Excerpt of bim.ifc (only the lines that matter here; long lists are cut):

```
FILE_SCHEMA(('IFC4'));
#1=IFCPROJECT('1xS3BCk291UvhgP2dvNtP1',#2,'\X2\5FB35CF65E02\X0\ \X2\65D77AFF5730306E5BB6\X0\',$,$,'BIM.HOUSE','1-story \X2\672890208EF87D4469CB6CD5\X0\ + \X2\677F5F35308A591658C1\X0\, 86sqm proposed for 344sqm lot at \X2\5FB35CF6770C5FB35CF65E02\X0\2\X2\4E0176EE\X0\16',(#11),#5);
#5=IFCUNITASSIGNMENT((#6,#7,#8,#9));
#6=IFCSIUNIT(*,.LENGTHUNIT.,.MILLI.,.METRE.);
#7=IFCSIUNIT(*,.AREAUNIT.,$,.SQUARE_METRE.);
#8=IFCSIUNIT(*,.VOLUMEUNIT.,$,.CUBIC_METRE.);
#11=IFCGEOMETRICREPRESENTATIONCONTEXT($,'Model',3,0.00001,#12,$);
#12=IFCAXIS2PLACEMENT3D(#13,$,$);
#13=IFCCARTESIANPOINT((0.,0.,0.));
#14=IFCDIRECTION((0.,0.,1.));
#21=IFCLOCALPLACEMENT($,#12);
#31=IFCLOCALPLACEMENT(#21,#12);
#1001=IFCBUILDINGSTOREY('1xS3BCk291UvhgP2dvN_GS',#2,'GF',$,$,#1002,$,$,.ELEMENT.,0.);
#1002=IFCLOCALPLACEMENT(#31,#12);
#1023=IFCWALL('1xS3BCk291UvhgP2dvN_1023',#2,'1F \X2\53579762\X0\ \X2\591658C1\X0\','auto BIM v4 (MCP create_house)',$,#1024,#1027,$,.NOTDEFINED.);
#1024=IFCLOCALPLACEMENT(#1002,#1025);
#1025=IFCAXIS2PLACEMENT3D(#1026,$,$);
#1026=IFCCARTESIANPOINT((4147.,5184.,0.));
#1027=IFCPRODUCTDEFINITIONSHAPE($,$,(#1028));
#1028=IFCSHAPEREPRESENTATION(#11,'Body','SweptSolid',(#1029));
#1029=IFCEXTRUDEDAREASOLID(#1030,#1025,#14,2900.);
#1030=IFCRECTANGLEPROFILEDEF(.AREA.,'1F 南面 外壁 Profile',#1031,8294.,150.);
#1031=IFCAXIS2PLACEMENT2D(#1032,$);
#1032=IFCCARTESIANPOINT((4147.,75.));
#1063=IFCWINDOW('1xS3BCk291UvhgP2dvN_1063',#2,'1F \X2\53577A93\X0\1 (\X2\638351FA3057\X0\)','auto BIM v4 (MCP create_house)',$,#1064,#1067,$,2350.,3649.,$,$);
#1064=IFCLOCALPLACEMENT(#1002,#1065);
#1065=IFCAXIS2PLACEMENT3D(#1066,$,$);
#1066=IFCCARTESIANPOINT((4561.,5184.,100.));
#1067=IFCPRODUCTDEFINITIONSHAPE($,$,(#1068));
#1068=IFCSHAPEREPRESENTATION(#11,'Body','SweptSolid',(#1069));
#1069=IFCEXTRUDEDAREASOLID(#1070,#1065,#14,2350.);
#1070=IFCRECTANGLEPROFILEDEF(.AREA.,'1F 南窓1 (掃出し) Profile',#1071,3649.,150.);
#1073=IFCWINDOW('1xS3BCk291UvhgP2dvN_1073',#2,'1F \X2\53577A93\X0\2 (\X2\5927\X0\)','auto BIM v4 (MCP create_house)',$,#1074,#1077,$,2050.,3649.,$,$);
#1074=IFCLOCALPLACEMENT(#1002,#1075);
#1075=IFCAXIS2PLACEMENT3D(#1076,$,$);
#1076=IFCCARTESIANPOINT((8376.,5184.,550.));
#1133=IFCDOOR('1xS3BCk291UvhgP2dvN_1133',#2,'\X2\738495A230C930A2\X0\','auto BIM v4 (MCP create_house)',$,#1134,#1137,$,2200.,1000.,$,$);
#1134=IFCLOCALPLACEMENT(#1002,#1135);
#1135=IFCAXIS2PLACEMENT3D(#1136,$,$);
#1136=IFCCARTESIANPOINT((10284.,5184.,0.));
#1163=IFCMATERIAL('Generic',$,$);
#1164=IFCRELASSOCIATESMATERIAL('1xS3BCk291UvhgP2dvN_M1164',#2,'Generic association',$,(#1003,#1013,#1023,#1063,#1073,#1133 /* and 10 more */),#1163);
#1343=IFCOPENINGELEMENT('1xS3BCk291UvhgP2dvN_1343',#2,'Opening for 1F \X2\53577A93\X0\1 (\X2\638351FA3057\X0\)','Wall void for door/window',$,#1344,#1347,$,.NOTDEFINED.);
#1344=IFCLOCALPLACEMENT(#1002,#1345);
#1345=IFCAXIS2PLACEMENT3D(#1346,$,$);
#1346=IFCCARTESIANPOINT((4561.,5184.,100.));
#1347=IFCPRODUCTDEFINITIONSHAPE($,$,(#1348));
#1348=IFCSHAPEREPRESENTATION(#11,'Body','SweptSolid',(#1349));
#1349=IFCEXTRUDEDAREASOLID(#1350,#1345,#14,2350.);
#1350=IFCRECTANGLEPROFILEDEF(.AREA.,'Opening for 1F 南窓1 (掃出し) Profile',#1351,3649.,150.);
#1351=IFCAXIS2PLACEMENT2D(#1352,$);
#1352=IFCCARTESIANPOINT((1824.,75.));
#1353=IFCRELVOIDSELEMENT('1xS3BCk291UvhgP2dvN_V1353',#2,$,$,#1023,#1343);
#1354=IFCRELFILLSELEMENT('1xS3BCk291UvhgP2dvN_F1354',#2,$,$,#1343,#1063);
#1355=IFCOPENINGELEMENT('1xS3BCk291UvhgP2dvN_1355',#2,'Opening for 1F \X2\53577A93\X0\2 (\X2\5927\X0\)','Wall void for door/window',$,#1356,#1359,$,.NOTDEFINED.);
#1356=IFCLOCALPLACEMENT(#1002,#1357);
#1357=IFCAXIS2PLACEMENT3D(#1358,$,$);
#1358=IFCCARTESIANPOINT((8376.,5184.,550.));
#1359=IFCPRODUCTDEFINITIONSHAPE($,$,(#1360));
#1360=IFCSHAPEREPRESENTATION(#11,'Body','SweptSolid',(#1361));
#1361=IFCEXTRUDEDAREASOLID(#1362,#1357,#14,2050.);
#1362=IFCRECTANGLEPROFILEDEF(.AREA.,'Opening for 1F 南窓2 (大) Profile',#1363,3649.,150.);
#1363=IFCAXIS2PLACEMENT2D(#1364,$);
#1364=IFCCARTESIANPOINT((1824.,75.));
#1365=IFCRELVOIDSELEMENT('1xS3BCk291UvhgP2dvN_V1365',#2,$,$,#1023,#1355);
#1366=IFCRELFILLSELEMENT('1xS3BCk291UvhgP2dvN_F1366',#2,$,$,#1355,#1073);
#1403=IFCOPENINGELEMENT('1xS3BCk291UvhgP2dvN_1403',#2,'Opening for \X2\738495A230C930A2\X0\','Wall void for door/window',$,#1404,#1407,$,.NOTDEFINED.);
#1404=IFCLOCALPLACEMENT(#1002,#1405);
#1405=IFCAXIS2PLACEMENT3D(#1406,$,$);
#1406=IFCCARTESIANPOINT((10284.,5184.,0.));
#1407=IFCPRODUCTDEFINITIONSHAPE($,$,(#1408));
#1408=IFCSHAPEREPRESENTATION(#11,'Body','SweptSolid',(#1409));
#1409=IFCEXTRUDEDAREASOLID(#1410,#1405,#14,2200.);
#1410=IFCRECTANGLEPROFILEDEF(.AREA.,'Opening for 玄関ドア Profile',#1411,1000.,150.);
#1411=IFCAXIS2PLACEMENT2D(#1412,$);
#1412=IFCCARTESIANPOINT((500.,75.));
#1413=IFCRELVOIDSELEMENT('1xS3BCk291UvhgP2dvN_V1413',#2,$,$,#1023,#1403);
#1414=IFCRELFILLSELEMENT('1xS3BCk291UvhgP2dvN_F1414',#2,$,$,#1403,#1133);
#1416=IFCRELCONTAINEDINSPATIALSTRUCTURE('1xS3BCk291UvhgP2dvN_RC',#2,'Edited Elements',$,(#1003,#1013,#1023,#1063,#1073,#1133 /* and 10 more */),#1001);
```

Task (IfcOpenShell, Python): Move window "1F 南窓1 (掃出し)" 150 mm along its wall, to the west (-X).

```python
import ifcopenshell
import ifcopenshell.api.geometry
import ifcopenshell.util.placement
import ifcopenshell.util.unit

model = ifcopenshell.open("bim.ifc")
unit_scale = ifcopenshell.util.unit.calculate_unit_scale(model)

window = model.by_guid("1xS3BCk291UvhgP2dvN_1063")
opening = window.FillsVoids[0].RelatingOpeningElement
wall = opening.VoidsElements[0].RelatingBuildingElement

wall_matrix = ifcopenshell.util.placement.get_local_placement(wall.ObjectPlacement)
shift = wall_matrix[:3, 0] * -0.15 / unit_scale
before = ifcopenshell.util.placement.get_local_placement(window.ObjectPlacement)[:3, 3].copy()

# The window is not placed relative to its opening, so move both.
for product in (opening, window):
    matrix = ifcopenshell.util.placement.get_local_placement(product.ObjectPlacement)
    matrix[:3, 3] += shift
    ifcopenshell.api.geometry.edit_object_placement(model, product=product, matrix=matrix, is_si=False)

after = ifcopenshell.util.placement.get_local_placement(window.ObjectPlacement)[:3, 3]
print("window moved by", (after - before).round(3) + 0.0)

model.write("bim_v2.ifc")
```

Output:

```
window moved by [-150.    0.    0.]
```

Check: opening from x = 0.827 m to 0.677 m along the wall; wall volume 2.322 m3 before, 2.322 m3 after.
